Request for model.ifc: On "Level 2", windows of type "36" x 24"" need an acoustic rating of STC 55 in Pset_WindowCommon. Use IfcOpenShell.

First a look at what the model holds.

```python
import ifcopenshell
import ifcopenshell.util.element

model = ifcopenshell.open("model.ifc")
print(model.schema)
storey = next(s for s in model.by_type("IfcBuildingStorey") if s.Name == "Level 2")
windows = [e for e in ifcopenshell.util.element.get_decomposition(storey) if e.is_a("IfcWindow")]
seen = {}
for e in windows:
    element_type = ifcopenshell.util.element.get_type(e)
    key = (element_type.Name if element_type != e and element_type else None, ifcopenshell.util.element.get_pset(e, "Pset_WindowCommon", "AcousticRating"))
    seen[key] = seen.get(key, 0) + 1
for (name, value), count in sorted(seen.items(), key=str):
    print(count, "x", name, "|", value)
```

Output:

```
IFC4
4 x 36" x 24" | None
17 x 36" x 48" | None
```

```python
import ifcopenshell
import ifcopenshell.api.pset
import ifcopenshell.util.element

model = ifcopenshell.open("model.ifc")

storey = next(s for s in model.by_type("IfcBuildingStorey") if s.Name == "Level 2")
windows = [e for e in ifcopenshell.util.element.get_decomposition(storey) if e.is_a("IfcWindow")]

count = 0
for e in windows:
    element_type = ifcopenshell.util.element.get_type(e)
    if element_type in (None, e) or element_type.Name != '36" x 24"':
        continue
    # add_pset returns the element's existing set when there is one.
    pset = ifcopenshell.api.pset.add_pset(model, product=e, name="Pset_WindowCommon")
    ifcopenshell.api.pset.edit_pset(model, pset=pset, properties={"AcousticRating": "STC 55"})
    count += 1

print(count, "windows updated")

model.write("model_edited.ifc")
```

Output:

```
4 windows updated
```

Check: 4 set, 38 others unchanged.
